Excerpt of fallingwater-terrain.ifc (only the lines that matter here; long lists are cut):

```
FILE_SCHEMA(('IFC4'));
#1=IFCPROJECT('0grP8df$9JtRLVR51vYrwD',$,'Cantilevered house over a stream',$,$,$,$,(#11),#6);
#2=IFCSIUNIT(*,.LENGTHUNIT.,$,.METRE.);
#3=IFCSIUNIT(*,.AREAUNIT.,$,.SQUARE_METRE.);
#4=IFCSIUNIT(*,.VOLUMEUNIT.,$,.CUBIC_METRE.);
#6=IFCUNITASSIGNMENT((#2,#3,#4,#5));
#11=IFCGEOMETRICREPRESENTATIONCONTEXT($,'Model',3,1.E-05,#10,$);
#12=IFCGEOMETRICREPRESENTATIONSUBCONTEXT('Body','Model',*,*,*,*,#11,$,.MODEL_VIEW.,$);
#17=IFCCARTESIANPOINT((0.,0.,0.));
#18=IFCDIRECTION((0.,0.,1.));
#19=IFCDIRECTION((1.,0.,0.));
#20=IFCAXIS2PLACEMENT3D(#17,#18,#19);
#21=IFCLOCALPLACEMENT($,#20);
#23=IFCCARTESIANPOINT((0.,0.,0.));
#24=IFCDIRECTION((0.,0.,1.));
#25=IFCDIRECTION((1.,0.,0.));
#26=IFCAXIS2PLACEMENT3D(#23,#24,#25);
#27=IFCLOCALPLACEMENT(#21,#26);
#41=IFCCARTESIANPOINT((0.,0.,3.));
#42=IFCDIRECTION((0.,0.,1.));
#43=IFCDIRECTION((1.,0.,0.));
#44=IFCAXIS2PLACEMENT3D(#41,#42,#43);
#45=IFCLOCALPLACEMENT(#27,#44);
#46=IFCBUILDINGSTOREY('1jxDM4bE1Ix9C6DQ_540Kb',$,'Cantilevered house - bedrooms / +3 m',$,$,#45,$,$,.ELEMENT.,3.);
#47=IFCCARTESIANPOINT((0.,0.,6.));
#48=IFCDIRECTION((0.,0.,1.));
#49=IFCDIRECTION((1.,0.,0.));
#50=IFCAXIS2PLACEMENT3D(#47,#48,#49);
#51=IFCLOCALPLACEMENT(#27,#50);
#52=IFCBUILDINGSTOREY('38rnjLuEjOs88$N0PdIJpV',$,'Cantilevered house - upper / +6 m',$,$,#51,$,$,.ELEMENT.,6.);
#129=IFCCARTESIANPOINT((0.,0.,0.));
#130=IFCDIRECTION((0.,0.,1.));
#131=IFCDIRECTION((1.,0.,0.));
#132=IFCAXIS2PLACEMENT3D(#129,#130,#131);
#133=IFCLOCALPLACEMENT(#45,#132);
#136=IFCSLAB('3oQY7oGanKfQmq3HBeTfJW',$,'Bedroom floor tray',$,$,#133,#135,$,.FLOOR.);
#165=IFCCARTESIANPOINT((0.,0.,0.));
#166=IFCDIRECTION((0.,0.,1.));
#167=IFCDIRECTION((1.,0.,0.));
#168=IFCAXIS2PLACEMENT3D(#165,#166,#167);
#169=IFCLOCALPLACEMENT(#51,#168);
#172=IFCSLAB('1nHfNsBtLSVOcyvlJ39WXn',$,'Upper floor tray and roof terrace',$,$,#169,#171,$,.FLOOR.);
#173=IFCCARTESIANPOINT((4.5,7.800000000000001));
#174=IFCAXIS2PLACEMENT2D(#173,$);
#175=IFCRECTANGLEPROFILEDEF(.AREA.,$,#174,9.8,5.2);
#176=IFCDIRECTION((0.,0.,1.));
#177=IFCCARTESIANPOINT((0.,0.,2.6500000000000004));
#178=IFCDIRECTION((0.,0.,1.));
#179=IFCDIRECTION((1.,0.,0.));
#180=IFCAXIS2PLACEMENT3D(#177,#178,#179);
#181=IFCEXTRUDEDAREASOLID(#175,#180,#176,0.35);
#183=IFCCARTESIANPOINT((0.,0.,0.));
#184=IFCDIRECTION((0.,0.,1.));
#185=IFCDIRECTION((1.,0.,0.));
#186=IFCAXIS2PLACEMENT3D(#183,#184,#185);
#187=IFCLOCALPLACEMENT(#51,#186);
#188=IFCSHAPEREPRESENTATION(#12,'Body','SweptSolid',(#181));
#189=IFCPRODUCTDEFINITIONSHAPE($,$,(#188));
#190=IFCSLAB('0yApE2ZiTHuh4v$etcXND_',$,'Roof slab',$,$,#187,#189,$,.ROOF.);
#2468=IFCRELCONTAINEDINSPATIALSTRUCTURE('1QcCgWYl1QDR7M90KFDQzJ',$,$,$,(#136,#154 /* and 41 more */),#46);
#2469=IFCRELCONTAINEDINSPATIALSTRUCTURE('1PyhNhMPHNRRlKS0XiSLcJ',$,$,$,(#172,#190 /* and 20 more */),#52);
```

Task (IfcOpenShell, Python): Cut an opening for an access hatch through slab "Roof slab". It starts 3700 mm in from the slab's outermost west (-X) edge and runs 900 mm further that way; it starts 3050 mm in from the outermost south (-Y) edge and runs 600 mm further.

```python
import numpy as np
import ifcopenshell
import ifcopenshell.api.feature
import ifcopenshell.api.geometry
import ifcopenshell.api.root
import ifcopenshell.geom
import ifcopenshell.util.placement
import ifcopenshell.util.representation
import ifcopenshell.util.shape
import ifcopenshell.util.unit

model = ifcopenshell.open("fallingwater-terrain.ifc")
unit_scale = ifcopenshell.util.unit.calculate_unit_scale(model)
settings = ifcopenshell.geom.settings()


def volume(element):
    """Net volume in cubic metres, openings subtracted."""
    shape = ifcopenshell.geom.create_shape(settings, element)
    return ifcopenshell.util.shape.get_volume(shape.geometry)


slab = model.by_id(190)
before = volume(slab)

# Extent in the slab's own axes, in metres. The edges named are its -X and -Y sides.
slab_shape = ifcopenshell.geom.create_shape(settings, slab)
vertices = ifcopenshell.util.shape.get_vertices(slab_shape.geometry)
x_min, y_min, bottom = vertices.min(axis=0)
top = vertices[:, 2].max()

opening = ifcopenshell.api.root.create_entity(model, ifc_class="IfcOpeningElement", name="Access hatch opening", predefined_type="OPENING")
context = ifcopenshell.util.representation.get_context(model, "Model", "Body", "MODEL_VIEW")
width, depth = 0.9, 0.6
outline = [(0.0, 0.0), (width, 0.0), (width, depth), (0.0, depth), (0.0, 0.0)]
# Overshoot both faces by 50 mm so the cut is clean.
shape = ifcopenshell.api.geometry.add_slab_representation(
    model, context=context, depth=top - bottom + 0.1, polyline=outline
)
ifcopenshell.api.geometry.assign_representation(model, product=opening, representation=shape)

matrix = ifcopenshell.util.placement.get_local_placement(slab.ObjectPlacement)
matrix[:, 3] = matrix @ np.append(np.array([x_min + 3.7, y_min + 3.05, bottom - 0.05]) / unit_scale, 1.0)
ifcopenshell.api.geometry.edit_object_placement(model, product=opening, matrix=matrix, is_si=False)
ifcopenshell.api.feature.add_feature(model, feature=opening, element=slab)

after = volume(slab)

print(f"slab volume {before:.3f} -> {after:.3f} m3")

model.write("fallingwater-terrain-out.ifc")
```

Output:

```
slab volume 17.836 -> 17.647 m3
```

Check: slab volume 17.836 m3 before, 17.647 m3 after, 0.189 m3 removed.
